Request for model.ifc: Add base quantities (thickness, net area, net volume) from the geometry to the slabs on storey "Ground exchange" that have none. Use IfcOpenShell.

First a look at what the model holds.

```python
import ifcopenshell
import ifcopenshell.util.element
import ifcopenshell.util.unit

model = ifcopenshell.open("model.ifc")
print(model.schema)
for unit_type in ("LENGTHUNIT", "AREAUNIT", "VOLUMEUNIT"):
    print(unit_type, ifcopenshell.util.unit.calculate_unit_scale(model, unit_type))
storey = next(s for s in model.by_type("IfcBuildingStorey") if s.Name == "Ground exchange")
slabs = [e for e in ifcopenshell.util.element.get_decomposition(storey) if e.is_a("IfcSlab")]
for e in sorted(slabs, key=lambda e: e.id()):
    print(e.id(), e.is_a(), e.Name, list(ifcopenshell.util.element.get_psets(e, qtos_only=True)), sep=" | ")
```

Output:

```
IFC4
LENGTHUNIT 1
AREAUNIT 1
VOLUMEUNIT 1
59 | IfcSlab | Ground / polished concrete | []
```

```python
import ifcopenshell
import ifcopenshell.api.pset
import ifcopenshell.geom
import ifcopenshell.util.element
import ifcopenshell.util.shape
import ifcopenshell.util.unit

model = ifcopenshell.open("model.ifc")
unit_scale = ifcopenshell.util.unit.calculate_unit_scale(model)
area_scale = ifcopenshell.util.unit.calculate_unit_scale(model, "AREAUNIT")
volume_scale = ifcopenshell.util.unit.calculate_unit_scale(model, "VOLUMEUNIT")
settings = ifcopenshell.geom.settings()

storey = next(s for s in model.by_type("IfcBuildingStorey") if s.Name == "Ground exchange")
slabs = [e for e in ifcopenshell.util.element.get_decomposition(storey) if e.is_a("IfcSlab")]

for e in sorted(slabs, key=lambda e: e.id()):
    if ifcopenshell.util.element.get_psets(e, qtos_only=True, should_inherit=False):
        continue
    # Geometry comes back in metres, in the element's own axes.
    shape = ifcopenshell.geom.create_shape(settings, e)
    values = {
        "Width": ifcopenshell.util.shape.get_z(shape.geometry) / unit_scale,
        "NetArea": ifcopenshell.util.shape.get_footprint_area(shape.geometry) / area_scale,
        "NetVolume": ifcopenshell.util.shape.get_volume(shape.geometry) / volume_scale,
    }
    qto = ifcopenshell.api.pset.add_qto(model, product=e, name="Qto_SlabBaseQuantities")
    ifcopenshell.api.pset.edit_qto(model, qto=qto, properties=values)
    print(e.id(), {k: round(v, 3) for k, v in values.items()})

model.write("model-out.ifc")
```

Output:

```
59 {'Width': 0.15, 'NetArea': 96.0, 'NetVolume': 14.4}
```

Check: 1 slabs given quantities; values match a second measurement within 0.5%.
